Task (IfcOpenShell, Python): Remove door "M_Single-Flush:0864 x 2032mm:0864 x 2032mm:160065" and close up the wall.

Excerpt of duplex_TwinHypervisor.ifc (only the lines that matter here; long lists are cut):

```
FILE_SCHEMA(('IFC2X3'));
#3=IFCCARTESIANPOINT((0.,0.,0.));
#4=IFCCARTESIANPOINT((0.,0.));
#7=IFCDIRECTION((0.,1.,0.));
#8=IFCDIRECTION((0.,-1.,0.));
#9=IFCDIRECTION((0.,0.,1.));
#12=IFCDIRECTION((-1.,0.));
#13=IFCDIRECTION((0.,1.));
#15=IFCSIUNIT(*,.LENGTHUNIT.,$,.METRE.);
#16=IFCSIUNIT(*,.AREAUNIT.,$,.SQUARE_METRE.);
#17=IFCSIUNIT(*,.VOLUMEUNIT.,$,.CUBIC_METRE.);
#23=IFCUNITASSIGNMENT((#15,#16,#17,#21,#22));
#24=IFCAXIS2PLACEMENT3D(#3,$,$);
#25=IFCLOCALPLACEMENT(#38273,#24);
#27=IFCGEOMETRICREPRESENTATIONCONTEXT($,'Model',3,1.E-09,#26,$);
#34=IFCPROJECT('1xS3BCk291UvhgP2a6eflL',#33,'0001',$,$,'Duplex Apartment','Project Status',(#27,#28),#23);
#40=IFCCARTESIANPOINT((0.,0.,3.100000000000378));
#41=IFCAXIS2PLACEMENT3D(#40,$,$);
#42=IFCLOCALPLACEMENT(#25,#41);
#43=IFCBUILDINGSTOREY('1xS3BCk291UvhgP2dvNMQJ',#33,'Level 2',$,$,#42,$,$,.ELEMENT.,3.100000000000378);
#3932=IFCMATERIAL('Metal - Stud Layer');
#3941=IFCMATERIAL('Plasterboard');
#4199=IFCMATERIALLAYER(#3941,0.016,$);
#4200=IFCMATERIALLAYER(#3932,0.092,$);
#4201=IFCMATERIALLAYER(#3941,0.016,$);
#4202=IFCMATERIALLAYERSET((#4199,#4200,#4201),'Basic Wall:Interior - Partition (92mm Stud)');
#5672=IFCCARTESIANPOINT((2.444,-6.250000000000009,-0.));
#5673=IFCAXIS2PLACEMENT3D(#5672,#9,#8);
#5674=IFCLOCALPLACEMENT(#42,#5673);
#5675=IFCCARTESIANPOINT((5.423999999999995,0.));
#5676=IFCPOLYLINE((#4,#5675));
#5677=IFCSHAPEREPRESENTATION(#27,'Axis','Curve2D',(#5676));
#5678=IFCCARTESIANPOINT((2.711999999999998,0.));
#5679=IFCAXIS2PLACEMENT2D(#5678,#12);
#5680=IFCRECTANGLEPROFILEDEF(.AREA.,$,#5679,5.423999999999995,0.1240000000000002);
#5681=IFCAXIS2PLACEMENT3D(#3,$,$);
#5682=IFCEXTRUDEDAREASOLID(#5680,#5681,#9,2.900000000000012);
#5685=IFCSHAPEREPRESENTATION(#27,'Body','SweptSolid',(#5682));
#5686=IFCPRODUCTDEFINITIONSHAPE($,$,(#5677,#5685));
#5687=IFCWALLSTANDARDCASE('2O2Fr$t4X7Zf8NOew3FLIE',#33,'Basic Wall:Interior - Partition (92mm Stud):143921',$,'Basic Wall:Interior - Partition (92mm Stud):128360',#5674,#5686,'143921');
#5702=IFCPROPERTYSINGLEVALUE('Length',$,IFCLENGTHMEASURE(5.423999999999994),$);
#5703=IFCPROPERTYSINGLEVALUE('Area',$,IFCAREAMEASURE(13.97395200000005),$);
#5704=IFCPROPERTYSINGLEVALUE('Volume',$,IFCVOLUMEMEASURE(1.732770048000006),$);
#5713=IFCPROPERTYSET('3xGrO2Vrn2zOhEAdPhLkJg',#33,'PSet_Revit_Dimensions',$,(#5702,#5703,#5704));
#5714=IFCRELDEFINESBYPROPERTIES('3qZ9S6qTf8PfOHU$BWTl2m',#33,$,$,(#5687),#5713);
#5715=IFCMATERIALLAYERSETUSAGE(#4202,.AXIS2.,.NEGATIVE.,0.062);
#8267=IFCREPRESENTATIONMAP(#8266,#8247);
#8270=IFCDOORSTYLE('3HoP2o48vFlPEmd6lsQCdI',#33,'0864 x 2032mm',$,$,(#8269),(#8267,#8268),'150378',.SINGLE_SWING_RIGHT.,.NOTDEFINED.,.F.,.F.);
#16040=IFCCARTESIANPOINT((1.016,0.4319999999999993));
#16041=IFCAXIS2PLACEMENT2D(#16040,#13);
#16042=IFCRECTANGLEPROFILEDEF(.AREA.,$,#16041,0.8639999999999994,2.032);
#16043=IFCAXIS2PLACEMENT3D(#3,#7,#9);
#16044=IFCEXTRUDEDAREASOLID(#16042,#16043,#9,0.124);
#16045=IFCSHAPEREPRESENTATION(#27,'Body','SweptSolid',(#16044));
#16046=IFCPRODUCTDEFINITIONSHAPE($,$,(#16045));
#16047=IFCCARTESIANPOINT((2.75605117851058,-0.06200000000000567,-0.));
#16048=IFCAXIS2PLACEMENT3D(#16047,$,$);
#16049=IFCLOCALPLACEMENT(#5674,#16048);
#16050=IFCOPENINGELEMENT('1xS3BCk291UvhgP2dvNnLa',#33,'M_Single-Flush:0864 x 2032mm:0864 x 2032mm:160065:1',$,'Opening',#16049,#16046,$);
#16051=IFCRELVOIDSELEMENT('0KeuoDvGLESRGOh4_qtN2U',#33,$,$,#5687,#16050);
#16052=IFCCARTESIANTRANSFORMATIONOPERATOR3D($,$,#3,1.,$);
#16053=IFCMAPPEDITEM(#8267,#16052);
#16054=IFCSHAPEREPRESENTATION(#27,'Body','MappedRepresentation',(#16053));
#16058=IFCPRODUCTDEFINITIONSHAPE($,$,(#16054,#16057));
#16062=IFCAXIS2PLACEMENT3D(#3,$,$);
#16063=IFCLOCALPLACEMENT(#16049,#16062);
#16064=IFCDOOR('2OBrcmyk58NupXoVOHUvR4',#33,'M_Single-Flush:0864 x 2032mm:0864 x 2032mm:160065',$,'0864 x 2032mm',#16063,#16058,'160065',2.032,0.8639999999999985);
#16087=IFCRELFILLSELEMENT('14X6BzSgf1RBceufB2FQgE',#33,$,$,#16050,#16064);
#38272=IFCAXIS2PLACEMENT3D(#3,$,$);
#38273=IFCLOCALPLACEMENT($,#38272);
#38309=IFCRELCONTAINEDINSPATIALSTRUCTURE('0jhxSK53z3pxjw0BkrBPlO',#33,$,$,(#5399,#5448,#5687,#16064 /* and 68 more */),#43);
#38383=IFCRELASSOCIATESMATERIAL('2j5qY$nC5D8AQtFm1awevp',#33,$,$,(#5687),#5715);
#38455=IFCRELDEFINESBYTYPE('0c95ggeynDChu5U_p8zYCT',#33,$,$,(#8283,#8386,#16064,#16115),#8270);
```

```python
import ifcopenshell
import ifcopenshell.api.feature
import ifcopenshell.api.pset
import ifcopenshell.api.root
import ifcopenshell.geom
import ifcopenshell.util.element
import ifcopenshell.util.shape
import ifcopenshell.util.unit

model = ifcopenshell.open("duplex_TwinHypervisor.ifc")
area_scale = ifcopenshell.util.unit.calculate_unit_scale(model, "AREAUNIT")
volume_scale = ifcopenshell.util.unit.calculate_unit_scale(model, "VOLUMEUNIT")
settings = ifcopenshell.geom.settings()


def volume(element):
    """Net volume in cubic metres, openings subtracted."""
    shape = ifcopenshell.geom.create_shape(settings, element)
    return ifcopenshell.util.shape.get_volume(shape.geometry)


door = model.by_guid("2OBrcmyk58NupXoVOHUvR4")
opening = door.FillsVoids[0].RelatingOpeningElement
wall = opening.VoidsElements[0].RelatingBuildingElement
before = volume(wall)

ifcopenshell.api.root.remove_product(model, product=door)
ifcopenshell.api.feature.remove_feature(model, feature=opening)

after = volume(wall)
thickness = 0.124  # wall thickness in metres

# Update the wall's stored quantities.
pset = model.by_id(ifcopenshell.util.element.get_pset(wall, "PSet_Revit_Dimensions", should_inherit=False)["id"])
ifcopenshell.api.pset.edit_pset(model, pset=pset, properties={
    "Area": model.create_entity("IfcAreaMeasure", after / thickness / area_scale),
    "Volume": model.create_entity("IfcVolumeMeasure", after / volume_scale),
})

print(f"wall volume {before:.3f} -> {after:.3f} m3")

model.write("duplex_TwinHypervisor_v2.ifc")
```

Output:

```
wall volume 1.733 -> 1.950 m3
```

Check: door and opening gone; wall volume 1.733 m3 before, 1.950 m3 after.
